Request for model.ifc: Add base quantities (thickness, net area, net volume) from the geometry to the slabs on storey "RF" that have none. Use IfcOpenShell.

First a look at what the model holds.

```python
import ifcopenshell
import ifcopenshell.util.element
import ifcopenshell.util.unit

model = ifcopenshell.open("model.ifc")
print(model.schema)
for unit_type in ("LENGTHUNIT", "AREAUNIT", "VOLUMEUNIT"):
    print(unit_type, ifcopenshell.util.unit.calculate_unit_scale(model, unit_type))
storey = next(s for s in model.by_type("IfcBuildingStorey") if s.Name == "RF")
slabs = [e for e in ifcopenshell.util.element.get_decomposition(storey) if e.is_a("IfcSlab")]
for e in sorted(slabs, key=lambda e: e.id()):
    print(e.id(), e.is_a(), e.Name, list(ifcopenshell.util.element.get_psets(e, qtos_only=True)), sep=" | ")
```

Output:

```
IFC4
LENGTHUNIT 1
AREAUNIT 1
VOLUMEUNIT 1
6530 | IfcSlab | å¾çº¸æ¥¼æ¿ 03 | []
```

```python
import ifcopenshell
import ifcopenshell.api.pset
import ifcopenshell.geom
import ifcopenshell.util.element
import ifcopenshell.util.shape
import ifcopenshell.util.unit

model = ifcopenshell.open("model.ifc")
unit_scale = ifcopenshell.util.unit.calculate_unit_scale(model)
area_scale = ifcopenshell.util.unit.calculate_unit_scale(model, "AREAUNIT")
volume_scale = ifcopenshell.util.unit.calculate_unit_scale(model, "VOLUMEUNIT")
settings = ifcopenshell.geom.settings()

storey = next(s for s in model.by_type("IfcBuildingStorey") if s.Name == "RF")
slabs = [e for e in ifcopenshell.util.element.get_decomposition(storey) if e.is_a("IfcSlab")]

for e in sorted(slabs, key=lambda e: e.id()):
    if ifcopenshell.util.element.get_psets(e, qtos_only=True, should_inherit=False):
        continue
    # Geometry comes back in metres, in the element's own axes.
    shape = ifcopenshell.geom.create_shape(settings, e)
    values = {
        "Width": ifcopenshell.util.shape.get_z(shape.geometry) / unit_scale,
        "NetArea": ifcopenshell.util.shape.get_footprint_area(shape.geometry) / area_scale,
        "NetVolume": ifcopenshell.util.shape.get_volume(shape.geometry) / volume_scale,
    }
    qto = ifcopenshell.api.pset.add_qto(model, product=e, name="Qto_SlabBaseQuantities")
    ifcopenshell.api.pset.edit_qto(model, qto=qto, properties=values)
    print(e.id(), {k: round(v, 3) for k, v in values.items()})

model.write("model-out.ifc")
```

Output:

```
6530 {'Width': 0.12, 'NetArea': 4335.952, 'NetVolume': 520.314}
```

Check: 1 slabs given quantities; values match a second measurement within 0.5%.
